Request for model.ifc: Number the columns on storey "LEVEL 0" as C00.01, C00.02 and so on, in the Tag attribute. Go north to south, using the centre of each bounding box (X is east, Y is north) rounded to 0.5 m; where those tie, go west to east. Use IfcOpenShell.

First a look at what the model holds.

```python
import ifcopenshell
import ifcopenshell.util.element
import ifcopenshell.util.placement

model = ifcopenshell.open("model.ifc")
print(model.schema)
storey = next(s for s in model.by_type("IfcBuildingStorey") if s.Name == "LEVEL 0")
columns = [e for e in ifcopenshell.util.element.get_decomposition(storey) if e.is_a("IfcColumn")]
for e in sorted(columns, key=lambda e: e.id()):
    origin = ifcopenshell.util.placement.get_local_placement(e.ObjectPlacement)[:3, 3]
    print(e.id(), e.Tag, e.Name, origin.round(2) + 0.0, sep=" | ")
```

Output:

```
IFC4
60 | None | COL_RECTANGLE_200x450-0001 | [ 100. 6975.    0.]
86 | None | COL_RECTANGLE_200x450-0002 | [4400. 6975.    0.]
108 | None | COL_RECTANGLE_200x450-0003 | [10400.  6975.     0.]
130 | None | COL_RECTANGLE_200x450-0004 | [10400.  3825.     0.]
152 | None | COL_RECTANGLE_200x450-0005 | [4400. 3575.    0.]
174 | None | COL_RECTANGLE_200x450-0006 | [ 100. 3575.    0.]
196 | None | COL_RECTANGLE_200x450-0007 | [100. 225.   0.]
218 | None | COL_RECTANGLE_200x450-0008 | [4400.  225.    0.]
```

```python
import ifcopenshell
import ifcopenshell.geom
import ifcopenshell.util.element
import ifcopenshell.util.shape

model = ifcopenshell.open("model.ifc")
settings = ifcopenshell.geom.settings()
settings.set("use-world-coords", True)


def centre(element):
    shape = ifcopenshell.geom.create_shape(settings, element)
    return ifcopenshell.util.shape.get_bbox_centroid(shape.geometry)


storey = next(s for s in model.by_type("IfcBuildingStorey") if s.Name == "LEVEL 0")
columns = [e for e in ifcopenshell.util.element.get_decomposition(storey) if e.is_a("IfcColumn")]

# Insertion points can sit at a corner or the storey origin, so sort by the geometry (in metres).
centres = {e: centre(e) for e in columns}
columns.sort(key=lambda e: (-round(centres[e][1] / 0.5), centres[e][0]))

for i, e in enumerate(columns, start=1):
    number = f"C00.{i:02d}"
    e.Tag = number
    print(e.id(), number)

model.write("model-out.ifc")
```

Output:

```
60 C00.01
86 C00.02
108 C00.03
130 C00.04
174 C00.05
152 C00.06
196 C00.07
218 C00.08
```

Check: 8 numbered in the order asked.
